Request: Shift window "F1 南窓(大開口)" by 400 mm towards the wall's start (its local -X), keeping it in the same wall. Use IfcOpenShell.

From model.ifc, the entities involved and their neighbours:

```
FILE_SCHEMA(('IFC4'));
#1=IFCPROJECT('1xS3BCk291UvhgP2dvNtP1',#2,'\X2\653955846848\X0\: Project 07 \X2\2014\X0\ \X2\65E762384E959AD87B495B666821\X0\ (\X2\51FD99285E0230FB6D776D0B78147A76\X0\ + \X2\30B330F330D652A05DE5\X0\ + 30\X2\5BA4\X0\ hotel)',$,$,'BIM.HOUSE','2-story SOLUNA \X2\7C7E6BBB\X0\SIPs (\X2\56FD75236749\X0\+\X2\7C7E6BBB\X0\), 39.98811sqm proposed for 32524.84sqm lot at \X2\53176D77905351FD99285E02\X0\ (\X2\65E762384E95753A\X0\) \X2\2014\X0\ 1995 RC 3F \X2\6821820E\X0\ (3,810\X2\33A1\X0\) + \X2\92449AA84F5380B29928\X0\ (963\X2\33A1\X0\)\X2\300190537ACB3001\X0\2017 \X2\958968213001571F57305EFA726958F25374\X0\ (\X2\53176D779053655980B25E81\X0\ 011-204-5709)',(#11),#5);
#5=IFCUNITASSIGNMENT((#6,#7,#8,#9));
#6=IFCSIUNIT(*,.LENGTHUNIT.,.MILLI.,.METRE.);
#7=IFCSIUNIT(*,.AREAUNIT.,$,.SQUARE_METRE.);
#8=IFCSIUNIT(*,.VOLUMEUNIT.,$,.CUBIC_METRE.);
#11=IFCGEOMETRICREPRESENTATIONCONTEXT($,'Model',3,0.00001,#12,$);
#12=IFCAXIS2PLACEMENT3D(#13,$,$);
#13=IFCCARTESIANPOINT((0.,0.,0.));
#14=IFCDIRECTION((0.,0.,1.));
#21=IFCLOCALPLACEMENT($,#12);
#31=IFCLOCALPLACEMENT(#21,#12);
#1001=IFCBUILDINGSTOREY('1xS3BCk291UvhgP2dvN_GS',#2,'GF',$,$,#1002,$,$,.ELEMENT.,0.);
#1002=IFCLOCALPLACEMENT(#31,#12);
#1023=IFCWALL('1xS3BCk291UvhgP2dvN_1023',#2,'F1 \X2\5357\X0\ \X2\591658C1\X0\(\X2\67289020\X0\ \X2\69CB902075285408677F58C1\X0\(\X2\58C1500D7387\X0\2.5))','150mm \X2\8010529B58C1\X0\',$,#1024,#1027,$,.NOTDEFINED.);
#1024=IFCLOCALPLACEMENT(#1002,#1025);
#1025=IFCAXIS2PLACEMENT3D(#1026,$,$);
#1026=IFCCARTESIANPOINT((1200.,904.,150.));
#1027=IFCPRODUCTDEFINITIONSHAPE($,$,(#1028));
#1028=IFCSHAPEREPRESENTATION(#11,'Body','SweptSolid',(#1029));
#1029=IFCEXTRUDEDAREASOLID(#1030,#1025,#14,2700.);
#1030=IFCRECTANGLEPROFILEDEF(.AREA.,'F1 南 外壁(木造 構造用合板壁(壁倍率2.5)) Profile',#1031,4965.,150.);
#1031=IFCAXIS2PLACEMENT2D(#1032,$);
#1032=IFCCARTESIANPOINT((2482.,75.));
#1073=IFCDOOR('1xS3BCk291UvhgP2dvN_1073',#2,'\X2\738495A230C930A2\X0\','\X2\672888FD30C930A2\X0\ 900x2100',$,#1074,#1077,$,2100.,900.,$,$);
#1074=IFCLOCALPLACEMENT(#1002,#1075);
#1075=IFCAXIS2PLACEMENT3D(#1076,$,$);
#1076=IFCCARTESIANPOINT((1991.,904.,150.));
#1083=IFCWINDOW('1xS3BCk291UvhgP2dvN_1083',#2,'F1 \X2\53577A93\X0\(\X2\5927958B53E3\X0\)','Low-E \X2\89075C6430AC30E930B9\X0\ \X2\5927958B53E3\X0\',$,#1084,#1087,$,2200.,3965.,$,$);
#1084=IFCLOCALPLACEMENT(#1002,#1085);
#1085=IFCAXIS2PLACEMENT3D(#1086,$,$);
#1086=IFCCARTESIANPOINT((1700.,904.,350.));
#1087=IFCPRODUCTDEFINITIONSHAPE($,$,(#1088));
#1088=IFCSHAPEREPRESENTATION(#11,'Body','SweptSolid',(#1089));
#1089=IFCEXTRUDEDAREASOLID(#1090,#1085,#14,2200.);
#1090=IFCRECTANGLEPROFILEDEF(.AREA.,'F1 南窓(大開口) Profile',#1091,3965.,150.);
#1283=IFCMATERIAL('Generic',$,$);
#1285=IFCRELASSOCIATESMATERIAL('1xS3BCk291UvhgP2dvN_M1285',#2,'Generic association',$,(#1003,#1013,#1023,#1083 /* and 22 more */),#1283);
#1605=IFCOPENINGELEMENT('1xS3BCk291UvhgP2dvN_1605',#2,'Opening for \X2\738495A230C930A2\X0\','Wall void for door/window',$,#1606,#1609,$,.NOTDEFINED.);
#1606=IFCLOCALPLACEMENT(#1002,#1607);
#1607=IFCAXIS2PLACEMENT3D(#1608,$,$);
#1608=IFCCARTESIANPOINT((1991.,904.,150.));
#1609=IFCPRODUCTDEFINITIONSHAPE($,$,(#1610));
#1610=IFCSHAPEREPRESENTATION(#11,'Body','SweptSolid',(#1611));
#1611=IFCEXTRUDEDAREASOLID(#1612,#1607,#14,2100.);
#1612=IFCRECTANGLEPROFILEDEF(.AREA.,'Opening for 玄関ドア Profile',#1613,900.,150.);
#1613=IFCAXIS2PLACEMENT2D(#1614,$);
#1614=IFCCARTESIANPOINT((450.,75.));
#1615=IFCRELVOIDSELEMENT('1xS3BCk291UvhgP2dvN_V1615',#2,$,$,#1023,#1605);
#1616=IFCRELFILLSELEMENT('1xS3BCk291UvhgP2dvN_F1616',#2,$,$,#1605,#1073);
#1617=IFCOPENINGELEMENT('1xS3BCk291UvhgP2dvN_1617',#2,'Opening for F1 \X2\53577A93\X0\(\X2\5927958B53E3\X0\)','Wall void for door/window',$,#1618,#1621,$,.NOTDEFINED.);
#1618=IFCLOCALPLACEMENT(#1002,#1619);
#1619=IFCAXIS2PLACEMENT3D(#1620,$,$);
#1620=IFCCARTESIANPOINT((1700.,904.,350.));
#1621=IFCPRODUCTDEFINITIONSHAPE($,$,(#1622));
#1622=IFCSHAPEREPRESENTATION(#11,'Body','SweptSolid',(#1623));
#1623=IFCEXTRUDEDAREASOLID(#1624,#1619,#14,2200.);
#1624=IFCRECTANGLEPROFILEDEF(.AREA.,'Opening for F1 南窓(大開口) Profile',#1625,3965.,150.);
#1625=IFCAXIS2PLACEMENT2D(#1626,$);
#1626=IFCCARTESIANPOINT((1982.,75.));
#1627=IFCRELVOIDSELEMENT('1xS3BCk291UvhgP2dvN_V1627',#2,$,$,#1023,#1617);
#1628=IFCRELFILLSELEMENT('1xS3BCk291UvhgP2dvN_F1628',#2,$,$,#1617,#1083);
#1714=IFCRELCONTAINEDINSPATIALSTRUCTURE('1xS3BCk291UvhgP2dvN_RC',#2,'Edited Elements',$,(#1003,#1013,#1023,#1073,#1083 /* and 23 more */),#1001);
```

```python
import ifcopenshell
import ifcopenshell.api.geometry
import ifcopenshell.util.placement
import ifcopenshell.util.unit

model = ifcopenshell.open("model.ifc")
unit_scale = ifcopenshell.util.unit.calculate_unit_scale(model)

window = model.by_guid("1xS3BCk291UvhgP2dvN_1083")
opening = window.FillsVoids[0].RelatingOpeningElement
wall = opening.VoidsElements[0].RelatingBuildingElement

wall_matrix = ifcopenshell.util.placement.get_local_placement(wall.ObjectPlacement)
shift = wall_matrix[:3, 0] * -0.4 / unit_scale
before = ifcopenshell.util.placement.get_local_placement(window.ObjectPlacement)[:3, 3].copy()

# The window is not placed relative to its opening, so move both.
for product in (opening, window):
    matrix = ifcopenshell.util.placement.get_local_placement(product.ObjectPlacement)
    matrix[:3, 3] += shift
    ifcopenshell.api.geometry.edit_object_placement(model, product=product, matrix=matrix, is_si=False)

after = ifcopenshell.util.placement.get_local_placement(window.ObjectPlacement)[:3, 3]
print("window moved by", (after - before).round(3) + 0.0)

model.write("model-out.ifc")
```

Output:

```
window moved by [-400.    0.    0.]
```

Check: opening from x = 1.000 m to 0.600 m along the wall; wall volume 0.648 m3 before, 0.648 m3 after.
